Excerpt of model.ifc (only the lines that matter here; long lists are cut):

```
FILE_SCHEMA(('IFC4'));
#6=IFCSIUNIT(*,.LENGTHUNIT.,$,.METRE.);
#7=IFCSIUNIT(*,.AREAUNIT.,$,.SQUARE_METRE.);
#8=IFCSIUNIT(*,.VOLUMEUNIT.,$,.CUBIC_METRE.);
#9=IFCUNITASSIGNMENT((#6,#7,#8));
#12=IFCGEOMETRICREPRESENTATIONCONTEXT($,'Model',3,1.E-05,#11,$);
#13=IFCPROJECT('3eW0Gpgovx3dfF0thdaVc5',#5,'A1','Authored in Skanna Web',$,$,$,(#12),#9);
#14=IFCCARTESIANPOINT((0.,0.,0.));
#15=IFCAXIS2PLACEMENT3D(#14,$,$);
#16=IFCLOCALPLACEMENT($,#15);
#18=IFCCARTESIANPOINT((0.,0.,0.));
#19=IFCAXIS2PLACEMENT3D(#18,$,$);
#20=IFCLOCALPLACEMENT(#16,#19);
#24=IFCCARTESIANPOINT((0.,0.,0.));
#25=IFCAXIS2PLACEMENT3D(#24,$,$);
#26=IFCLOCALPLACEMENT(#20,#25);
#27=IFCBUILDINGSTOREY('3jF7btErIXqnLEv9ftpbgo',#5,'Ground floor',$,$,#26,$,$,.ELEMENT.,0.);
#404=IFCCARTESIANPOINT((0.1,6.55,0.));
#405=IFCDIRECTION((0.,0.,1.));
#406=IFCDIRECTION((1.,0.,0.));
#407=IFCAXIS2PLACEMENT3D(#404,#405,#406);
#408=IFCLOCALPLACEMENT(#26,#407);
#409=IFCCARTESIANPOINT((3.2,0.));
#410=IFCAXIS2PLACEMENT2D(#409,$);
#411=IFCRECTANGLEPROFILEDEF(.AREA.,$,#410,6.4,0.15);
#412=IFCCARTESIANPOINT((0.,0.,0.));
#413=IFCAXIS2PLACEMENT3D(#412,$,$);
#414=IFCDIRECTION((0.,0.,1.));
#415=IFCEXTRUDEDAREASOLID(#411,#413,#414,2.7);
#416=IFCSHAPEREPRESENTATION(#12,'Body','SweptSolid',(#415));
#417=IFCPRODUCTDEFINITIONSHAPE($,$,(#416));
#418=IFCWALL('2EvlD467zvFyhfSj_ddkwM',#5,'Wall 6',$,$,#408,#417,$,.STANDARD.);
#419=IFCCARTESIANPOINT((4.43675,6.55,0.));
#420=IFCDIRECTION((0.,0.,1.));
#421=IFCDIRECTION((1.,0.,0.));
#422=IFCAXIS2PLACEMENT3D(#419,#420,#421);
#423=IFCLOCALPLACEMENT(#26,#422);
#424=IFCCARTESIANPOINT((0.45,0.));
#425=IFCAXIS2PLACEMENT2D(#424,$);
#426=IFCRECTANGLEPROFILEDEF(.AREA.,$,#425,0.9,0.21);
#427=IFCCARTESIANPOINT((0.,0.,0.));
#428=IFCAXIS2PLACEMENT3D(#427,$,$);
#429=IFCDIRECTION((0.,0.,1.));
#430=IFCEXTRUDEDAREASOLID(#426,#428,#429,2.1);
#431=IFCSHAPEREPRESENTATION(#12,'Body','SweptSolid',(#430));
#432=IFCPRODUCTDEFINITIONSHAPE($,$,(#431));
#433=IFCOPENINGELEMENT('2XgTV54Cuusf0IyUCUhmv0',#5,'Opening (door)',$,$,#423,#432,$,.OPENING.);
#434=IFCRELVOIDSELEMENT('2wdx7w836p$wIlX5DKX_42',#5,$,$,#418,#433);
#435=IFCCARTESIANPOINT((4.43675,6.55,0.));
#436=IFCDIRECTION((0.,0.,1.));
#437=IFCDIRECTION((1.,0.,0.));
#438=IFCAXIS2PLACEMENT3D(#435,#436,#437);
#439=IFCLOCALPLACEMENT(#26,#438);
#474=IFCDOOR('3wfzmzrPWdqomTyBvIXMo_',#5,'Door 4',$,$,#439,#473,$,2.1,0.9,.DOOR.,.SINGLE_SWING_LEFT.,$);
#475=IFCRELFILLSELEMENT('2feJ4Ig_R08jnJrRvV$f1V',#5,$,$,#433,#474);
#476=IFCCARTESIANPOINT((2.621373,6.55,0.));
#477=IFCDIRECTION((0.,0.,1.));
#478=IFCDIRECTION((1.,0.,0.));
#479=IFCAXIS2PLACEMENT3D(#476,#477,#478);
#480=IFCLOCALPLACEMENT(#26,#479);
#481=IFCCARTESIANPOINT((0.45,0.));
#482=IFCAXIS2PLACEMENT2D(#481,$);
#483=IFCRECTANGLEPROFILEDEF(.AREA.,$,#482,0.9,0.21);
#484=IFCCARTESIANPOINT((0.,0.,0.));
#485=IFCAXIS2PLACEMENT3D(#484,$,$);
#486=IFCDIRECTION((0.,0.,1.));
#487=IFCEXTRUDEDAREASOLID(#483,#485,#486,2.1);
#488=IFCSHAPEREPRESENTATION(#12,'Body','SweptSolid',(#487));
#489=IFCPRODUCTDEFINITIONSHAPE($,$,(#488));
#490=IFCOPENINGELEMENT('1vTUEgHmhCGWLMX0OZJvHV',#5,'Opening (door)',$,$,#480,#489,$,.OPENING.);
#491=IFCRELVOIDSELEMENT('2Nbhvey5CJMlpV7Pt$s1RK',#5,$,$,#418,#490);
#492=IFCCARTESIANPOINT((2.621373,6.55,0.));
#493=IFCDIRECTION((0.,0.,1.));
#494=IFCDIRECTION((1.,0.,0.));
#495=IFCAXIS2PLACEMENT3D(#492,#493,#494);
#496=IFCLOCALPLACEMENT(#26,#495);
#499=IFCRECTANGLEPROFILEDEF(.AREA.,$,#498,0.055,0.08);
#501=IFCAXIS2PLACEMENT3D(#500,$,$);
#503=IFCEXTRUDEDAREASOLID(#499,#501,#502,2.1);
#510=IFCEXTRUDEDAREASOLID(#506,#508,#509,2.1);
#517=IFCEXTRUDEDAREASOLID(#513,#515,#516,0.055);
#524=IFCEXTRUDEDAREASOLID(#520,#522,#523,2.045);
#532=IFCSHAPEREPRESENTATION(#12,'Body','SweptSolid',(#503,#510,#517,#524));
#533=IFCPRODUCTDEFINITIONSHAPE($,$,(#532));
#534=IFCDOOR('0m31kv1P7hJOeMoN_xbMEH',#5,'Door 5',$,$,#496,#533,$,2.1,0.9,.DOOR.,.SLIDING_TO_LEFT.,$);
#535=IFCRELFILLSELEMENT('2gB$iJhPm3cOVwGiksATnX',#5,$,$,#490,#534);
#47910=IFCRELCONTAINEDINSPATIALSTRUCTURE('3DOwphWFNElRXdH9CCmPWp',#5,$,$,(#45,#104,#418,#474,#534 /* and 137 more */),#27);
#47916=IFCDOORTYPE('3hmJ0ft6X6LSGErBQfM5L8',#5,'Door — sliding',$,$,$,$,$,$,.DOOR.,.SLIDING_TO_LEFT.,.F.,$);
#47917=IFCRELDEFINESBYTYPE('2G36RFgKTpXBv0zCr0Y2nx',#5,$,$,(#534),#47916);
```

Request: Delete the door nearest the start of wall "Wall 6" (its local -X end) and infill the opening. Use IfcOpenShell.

```python
import ifcopenshell
import ifcopenshell.api.feature
import ifcopenshell.api.root
import ifcopenshell.geom
import ifcopenshell.util.shape

model = ifcopenshell.open("model.ifc")
settings = ifcopenshell.geom.settings()


def volume(element):
    """Net volume in cubic metres, openings subtracted."""
    shape = ifcopenshell.geom.create_shape(settings, element)
    return ifcopenshell.util.shape.get_volume(shape.geometry)


door = model.by_id(534)
opening = door.FillsVoids[0].RelatingOpeningElement
wall = opening.VoidsElements[0].RelatingBuildingElement
before = volume(wall)

ifcopenshell.api.root.remove_product(model, product=door)
ifcopenshell.api.feature.remove_feature(model, feature=opening)

after = volume(wall)

print(f"wall volume {before:.3f} -> {after:.3f} m3")

model.write("model_updated.ifc")
```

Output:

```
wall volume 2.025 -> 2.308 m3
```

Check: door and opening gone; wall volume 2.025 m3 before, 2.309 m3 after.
